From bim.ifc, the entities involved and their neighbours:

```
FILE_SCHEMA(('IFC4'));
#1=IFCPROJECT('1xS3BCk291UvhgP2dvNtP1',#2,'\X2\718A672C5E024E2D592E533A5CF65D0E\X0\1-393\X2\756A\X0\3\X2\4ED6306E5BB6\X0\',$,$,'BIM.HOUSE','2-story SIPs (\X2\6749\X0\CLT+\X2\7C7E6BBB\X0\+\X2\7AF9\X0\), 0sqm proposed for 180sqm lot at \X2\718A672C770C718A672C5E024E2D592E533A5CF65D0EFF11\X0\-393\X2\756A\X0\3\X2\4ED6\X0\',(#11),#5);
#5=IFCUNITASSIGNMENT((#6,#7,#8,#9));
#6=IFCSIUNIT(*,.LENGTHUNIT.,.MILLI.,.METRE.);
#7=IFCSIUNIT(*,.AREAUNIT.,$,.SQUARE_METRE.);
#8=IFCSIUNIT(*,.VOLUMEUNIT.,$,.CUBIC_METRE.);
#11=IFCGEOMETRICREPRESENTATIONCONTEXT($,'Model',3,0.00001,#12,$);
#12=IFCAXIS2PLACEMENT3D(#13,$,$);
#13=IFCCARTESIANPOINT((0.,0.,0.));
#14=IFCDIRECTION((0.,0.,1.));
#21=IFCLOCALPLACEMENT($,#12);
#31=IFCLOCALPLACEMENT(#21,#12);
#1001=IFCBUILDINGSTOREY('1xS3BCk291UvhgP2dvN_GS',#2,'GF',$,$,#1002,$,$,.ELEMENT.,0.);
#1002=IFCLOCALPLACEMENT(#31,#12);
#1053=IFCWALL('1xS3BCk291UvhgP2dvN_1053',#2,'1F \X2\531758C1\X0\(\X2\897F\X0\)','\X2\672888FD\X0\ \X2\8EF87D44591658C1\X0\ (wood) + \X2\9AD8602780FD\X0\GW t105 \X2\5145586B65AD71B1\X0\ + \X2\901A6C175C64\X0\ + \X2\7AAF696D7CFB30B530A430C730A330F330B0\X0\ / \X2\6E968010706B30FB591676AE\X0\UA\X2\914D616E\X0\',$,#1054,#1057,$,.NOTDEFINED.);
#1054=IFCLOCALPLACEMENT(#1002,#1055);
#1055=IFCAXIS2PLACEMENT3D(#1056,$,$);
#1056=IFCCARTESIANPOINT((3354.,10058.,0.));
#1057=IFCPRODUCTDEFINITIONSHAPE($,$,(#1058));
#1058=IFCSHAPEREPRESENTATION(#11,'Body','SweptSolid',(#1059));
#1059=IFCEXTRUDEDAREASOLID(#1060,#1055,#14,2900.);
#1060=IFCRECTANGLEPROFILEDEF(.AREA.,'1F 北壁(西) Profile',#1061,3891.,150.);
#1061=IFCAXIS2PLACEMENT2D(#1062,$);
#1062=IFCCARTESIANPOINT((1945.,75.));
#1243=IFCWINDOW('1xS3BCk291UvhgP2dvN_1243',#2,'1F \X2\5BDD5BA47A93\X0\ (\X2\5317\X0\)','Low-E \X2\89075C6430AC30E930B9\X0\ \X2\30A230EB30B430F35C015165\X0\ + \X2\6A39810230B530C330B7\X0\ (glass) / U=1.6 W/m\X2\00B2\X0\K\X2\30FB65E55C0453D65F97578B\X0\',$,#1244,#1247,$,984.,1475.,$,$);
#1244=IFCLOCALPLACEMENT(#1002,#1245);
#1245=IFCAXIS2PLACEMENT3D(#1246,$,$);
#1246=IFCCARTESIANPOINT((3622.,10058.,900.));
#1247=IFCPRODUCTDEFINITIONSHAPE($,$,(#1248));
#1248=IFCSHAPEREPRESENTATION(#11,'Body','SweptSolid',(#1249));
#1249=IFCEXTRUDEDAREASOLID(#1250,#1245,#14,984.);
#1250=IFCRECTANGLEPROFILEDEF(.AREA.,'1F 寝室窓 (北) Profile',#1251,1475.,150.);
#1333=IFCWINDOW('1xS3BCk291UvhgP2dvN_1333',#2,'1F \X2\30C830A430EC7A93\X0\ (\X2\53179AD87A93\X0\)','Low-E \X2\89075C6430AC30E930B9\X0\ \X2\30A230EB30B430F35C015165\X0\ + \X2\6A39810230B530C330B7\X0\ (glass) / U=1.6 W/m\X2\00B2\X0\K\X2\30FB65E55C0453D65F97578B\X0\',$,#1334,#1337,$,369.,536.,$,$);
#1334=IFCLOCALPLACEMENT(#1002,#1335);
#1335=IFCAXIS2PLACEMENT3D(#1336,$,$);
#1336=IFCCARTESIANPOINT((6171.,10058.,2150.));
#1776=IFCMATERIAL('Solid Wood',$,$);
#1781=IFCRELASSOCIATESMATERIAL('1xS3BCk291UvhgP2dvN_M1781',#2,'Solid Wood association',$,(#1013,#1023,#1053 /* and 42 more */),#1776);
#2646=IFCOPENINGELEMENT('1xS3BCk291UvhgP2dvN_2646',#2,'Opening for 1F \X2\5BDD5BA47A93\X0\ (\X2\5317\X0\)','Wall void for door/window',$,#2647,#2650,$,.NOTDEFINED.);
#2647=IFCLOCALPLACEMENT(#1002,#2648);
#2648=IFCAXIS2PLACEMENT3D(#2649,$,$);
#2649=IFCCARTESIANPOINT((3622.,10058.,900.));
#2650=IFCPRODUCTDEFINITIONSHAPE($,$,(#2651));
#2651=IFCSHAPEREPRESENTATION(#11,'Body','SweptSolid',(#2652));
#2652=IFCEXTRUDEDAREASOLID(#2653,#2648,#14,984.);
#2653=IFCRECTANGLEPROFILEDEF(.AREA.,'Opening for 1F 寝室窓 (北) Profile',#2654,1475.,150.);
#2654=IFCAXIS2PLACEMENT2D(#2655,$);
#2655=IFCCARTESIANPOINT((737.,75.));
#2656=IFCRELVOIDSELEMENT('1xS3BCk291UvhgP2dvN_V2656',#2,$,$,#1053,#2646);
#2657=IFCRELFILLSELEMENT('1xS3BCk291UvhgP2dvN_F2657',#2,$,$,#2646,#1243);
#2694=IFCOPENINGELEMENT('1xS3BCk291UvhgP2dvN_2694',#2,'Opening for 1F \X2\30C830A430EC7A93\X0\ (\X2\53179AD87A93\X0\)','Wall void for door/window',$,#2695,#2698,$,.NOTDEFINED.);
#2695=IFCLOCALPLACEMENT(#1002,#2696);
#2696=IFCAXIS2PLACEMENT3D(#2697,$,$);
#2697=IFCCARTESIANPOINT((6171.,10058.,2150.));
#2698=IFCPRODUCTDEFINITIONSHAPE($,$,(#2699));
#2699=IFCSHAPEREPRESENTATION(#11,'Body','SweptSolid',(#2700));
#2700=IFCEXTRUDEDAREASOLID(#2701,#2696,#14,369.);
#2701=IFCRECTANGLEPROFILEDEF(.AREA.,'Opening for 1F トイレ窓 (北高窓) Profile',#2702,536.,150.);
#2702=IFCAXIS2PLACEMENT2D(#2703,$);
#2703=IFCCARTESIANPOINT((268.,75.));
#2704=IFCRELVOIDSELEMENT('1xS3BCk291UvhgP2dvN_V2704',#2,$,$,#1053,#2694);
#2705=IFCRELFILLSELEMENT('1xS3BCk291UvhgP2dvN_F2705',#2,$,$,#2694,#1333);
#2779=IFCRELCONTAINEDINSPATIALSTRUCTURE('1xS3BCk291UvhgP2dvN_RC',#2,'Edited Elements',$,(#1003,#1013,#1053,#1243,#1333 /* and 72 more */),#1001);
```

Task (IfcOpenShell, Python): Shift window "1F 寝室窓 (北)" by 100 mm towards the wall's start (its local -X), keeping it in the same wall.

```python
import ifcopenshell
import ifcopenshell.api.geometry
import ifcopenshell.util.placement

model = ifcopenshell.open("bim.ifc")

window = model.by_guid("1xS3BCk291UvhgP2dvN_1243")
opening = window.FillsVoids[0].RelatingOpeningElement
wall = opening.VoidsElements[0].RelatingBuildingElement

wall_matrix = ifcopenshell.util.placement.get_local_placement(wall.ObjectPlacement)
shift = wall_matrix[:3, 0] * -100.0
before = ifcopenshell.util.placement.get_local_placement(window.ObjectPlacement)[:3, 3].copy()

# The window is not placed relative to its opening, so move both.
for product in (opening, window):
    matrix = ifcopenshell.util.placement.get_local_placement(product.ObjectPlacement)
    matrix[:3, 3] += shift
    ifcopenshell.api.geometry.edit_object_placement(model, product=product, matrix=matrix, is_si=False)

after = ifcopenshell.util.placement.get_local_placement(window.ObjectPlacement)[:3, 3]
print("window moved by", (after - before).round(3) + 0.0)

model.write("bim_rev.ifc")
```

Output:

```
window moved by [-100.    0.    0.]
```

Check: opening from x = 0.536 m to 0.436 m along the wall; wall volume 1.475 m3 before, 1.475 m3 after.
